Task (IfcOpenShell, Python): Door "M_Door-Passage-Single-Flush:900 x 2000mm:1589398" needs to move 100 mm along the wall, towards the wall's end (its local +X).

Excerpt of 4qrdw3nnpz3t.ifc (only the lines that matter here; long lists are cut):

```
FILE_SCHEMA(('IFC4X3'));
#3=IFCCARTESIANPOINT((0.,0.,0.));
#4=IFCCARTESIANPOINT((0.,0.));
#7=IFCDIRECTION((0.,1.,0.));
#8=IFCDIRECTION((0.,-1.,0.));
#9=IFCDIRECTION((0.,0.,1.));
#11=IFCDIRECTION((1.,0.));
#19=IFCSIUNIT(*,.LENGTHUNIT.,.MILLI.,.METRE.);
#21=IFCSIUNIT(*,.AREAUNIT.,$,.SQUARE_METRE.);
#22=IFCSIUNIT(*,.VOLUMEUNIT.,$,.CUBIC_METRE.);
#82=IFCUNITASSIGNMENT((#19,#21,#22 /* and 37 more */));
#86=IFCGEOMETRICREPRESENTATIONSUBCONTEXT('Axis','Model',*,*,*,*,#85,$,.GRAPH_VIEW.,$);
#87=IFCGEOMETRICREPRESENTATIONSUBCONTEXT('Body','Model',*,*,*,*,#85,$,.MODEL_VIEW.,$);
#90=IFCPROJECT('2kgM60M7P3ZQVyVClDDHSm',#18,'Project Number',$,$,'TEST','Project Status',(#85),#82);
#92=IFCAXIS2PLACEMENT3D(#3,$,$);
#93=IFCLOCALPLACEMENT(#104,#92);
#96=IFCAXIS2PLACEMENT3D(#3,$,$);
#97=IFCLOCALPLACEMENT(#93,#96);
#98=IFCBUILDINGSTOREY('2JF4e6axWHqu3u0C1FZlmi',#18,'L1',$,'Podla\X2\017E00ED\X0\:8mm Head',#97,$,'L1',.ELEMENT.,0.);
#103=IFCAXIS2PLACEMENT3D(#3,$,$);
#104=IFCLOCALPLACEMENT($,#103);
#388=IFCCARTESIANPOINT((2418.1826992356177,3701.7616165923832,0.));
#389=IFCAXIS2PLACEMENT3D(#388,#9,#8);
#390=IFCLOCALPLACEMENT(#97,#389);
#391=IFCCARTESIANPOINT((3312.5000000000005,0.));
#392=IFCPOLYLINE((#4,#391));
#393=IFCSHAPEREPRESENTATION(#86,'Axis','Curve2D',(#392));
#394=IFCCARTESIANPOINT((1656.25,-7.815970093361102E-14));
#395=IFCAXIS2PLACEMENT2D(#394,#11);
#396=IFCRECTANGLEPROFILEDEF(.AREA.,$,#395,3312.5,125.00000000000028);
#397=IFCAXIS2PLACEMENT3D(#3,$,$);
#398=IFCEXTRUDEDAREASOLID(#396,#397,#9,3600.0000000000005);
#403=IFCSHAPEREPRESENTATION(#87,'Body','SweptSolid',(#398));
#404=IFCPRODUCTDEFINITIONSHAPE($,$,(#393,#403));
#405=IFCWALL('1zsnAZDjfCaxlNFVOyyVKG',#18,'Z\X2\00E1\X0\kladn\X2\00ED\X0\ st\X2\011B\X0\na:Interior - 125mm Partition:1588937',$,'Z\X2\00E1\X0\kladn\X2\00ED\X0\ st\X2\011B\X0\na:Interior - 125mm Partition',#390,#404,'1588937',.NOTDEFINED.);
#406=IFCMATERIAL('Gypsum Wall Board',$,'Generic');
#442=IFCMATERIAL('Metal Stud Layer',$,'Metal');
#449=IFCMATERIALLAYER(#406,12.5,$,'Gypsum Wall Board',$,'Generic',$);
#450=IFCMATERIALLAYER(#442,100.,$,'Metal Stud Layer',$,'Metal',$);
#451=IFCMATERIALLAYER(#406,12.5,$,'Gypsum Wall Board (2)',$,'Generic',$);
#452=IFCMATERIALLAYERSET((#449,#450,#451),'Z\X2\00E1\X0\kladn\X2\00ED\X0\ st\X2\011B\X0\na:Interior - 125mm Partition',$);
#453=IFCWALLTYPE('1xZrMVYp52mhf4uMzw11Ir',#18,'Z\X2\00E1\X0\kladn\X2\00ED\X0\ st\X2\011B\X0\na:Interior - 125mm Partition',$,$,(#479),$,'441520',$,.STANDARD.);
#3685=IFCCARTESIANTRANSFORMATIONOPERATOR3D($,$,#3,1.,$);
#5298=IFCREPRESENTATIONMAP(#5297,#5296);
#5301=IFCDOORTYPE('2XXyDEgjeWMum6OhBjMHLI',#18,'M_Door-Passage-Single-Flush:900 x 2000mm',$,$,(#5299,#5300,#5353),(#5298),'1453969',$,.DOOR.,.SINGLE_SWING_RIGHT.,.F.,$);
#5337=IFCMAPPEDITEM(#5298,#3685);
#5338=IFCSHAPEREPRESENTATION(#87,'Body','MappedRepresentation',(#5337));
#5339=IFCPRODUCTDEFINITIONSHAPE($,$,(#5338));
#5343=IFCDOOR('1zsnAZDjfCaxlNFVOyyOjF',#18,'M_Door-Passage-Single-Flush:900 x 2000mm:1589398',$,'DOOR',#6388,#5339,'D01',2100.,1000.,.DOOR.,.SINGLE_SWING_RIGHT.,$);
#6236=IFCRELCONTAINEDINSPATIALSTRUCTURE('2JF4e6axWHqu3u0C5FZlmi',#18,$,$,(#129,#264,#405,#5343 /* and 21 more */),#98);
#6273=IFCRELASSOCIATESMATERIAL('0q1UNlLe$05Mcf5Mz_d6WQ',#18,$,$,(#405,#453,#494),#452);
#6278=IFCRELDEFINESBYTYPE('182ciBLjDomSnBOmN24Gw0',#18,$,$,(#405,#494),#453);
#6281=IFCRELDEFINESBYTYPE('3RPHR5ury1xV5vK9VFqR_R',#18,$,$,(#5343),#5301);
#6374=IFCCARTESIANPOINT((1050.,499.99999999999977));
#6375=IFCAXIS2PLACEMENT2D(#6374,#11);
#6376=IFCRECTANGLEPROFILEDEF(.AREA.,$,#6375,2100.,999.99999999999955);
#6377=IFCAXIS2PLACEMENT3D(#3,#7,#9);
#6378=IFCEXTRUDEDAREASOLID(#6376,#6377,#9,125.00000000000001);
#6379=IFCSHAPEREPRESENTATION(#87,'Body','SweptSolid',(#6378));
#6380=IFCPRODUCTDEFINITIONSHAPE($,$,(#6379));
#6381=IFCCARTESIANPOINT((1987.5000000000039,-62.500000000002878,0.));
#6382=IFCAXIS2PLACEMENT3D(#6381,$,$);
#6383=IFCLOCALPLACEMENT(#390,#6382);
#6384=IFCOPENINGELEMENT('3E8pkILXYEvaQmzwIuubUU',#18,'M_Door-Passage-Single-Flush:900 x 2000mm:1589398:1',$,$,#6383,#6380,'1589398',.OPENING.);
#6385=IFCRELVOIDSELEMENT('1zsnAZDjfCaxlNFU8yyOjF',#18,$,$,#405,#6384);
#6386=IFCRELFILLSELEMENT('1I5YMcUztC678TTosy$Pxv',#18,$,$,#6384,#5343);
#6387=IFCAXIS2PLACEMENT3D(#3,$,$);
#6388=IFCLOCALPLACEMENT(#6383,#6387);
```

```python
import ifcopenshell
import ifcopenshell.api.geometry
import ifcopenshell.util.placement
import ifcopenshell.util.unit

model = ifcopenshell.open("4qrdw3nnpz3t.ifc")
unit_scale = ifcopenshell.util.unit.calculate_unit_scale(model)

door = model.by_guid("1zsnAZDjfCaxlNFVOyyOjF")
opening = door.FillsVoids[0].RelatingOpeningElement
wall = opening.VoidsElements[0].RelatingBuildingElement

wall_matrix = ifcopenshell.util.placement.get_local_placement(wall.ObjectPlacement)
shift = wall_matrix[:3, 0] * 0.1 / unit_scale
before = ifcopenshell.util.placement.get_local_placement(door.ObjectPlacement)[:3, 3].copy()

# The door is placed relative to its opening, so it follows when the opening moves.
matrix = ifcopenshell.util.placement.get_local_placement(opening.ObjectPlacement)
matrix[:3, 3] += shift
ifcopenshell.api.geometry.edit_object_placement(
    model, product=opening, matrix=matrix, is_si=False, should_transform_children=True
)

after = ifcopenshell.util.placement.get_local_placement(door.ObjectPlacement)[:3, 3]
print("door moved by", (after - before).round(3) + 0.0)

model.write("4qrdw3nnpz3t_v2.ifc")
```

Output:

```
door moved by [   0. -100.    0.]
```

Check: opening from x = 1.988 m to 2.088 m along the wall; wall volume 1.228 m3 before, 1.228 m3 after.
